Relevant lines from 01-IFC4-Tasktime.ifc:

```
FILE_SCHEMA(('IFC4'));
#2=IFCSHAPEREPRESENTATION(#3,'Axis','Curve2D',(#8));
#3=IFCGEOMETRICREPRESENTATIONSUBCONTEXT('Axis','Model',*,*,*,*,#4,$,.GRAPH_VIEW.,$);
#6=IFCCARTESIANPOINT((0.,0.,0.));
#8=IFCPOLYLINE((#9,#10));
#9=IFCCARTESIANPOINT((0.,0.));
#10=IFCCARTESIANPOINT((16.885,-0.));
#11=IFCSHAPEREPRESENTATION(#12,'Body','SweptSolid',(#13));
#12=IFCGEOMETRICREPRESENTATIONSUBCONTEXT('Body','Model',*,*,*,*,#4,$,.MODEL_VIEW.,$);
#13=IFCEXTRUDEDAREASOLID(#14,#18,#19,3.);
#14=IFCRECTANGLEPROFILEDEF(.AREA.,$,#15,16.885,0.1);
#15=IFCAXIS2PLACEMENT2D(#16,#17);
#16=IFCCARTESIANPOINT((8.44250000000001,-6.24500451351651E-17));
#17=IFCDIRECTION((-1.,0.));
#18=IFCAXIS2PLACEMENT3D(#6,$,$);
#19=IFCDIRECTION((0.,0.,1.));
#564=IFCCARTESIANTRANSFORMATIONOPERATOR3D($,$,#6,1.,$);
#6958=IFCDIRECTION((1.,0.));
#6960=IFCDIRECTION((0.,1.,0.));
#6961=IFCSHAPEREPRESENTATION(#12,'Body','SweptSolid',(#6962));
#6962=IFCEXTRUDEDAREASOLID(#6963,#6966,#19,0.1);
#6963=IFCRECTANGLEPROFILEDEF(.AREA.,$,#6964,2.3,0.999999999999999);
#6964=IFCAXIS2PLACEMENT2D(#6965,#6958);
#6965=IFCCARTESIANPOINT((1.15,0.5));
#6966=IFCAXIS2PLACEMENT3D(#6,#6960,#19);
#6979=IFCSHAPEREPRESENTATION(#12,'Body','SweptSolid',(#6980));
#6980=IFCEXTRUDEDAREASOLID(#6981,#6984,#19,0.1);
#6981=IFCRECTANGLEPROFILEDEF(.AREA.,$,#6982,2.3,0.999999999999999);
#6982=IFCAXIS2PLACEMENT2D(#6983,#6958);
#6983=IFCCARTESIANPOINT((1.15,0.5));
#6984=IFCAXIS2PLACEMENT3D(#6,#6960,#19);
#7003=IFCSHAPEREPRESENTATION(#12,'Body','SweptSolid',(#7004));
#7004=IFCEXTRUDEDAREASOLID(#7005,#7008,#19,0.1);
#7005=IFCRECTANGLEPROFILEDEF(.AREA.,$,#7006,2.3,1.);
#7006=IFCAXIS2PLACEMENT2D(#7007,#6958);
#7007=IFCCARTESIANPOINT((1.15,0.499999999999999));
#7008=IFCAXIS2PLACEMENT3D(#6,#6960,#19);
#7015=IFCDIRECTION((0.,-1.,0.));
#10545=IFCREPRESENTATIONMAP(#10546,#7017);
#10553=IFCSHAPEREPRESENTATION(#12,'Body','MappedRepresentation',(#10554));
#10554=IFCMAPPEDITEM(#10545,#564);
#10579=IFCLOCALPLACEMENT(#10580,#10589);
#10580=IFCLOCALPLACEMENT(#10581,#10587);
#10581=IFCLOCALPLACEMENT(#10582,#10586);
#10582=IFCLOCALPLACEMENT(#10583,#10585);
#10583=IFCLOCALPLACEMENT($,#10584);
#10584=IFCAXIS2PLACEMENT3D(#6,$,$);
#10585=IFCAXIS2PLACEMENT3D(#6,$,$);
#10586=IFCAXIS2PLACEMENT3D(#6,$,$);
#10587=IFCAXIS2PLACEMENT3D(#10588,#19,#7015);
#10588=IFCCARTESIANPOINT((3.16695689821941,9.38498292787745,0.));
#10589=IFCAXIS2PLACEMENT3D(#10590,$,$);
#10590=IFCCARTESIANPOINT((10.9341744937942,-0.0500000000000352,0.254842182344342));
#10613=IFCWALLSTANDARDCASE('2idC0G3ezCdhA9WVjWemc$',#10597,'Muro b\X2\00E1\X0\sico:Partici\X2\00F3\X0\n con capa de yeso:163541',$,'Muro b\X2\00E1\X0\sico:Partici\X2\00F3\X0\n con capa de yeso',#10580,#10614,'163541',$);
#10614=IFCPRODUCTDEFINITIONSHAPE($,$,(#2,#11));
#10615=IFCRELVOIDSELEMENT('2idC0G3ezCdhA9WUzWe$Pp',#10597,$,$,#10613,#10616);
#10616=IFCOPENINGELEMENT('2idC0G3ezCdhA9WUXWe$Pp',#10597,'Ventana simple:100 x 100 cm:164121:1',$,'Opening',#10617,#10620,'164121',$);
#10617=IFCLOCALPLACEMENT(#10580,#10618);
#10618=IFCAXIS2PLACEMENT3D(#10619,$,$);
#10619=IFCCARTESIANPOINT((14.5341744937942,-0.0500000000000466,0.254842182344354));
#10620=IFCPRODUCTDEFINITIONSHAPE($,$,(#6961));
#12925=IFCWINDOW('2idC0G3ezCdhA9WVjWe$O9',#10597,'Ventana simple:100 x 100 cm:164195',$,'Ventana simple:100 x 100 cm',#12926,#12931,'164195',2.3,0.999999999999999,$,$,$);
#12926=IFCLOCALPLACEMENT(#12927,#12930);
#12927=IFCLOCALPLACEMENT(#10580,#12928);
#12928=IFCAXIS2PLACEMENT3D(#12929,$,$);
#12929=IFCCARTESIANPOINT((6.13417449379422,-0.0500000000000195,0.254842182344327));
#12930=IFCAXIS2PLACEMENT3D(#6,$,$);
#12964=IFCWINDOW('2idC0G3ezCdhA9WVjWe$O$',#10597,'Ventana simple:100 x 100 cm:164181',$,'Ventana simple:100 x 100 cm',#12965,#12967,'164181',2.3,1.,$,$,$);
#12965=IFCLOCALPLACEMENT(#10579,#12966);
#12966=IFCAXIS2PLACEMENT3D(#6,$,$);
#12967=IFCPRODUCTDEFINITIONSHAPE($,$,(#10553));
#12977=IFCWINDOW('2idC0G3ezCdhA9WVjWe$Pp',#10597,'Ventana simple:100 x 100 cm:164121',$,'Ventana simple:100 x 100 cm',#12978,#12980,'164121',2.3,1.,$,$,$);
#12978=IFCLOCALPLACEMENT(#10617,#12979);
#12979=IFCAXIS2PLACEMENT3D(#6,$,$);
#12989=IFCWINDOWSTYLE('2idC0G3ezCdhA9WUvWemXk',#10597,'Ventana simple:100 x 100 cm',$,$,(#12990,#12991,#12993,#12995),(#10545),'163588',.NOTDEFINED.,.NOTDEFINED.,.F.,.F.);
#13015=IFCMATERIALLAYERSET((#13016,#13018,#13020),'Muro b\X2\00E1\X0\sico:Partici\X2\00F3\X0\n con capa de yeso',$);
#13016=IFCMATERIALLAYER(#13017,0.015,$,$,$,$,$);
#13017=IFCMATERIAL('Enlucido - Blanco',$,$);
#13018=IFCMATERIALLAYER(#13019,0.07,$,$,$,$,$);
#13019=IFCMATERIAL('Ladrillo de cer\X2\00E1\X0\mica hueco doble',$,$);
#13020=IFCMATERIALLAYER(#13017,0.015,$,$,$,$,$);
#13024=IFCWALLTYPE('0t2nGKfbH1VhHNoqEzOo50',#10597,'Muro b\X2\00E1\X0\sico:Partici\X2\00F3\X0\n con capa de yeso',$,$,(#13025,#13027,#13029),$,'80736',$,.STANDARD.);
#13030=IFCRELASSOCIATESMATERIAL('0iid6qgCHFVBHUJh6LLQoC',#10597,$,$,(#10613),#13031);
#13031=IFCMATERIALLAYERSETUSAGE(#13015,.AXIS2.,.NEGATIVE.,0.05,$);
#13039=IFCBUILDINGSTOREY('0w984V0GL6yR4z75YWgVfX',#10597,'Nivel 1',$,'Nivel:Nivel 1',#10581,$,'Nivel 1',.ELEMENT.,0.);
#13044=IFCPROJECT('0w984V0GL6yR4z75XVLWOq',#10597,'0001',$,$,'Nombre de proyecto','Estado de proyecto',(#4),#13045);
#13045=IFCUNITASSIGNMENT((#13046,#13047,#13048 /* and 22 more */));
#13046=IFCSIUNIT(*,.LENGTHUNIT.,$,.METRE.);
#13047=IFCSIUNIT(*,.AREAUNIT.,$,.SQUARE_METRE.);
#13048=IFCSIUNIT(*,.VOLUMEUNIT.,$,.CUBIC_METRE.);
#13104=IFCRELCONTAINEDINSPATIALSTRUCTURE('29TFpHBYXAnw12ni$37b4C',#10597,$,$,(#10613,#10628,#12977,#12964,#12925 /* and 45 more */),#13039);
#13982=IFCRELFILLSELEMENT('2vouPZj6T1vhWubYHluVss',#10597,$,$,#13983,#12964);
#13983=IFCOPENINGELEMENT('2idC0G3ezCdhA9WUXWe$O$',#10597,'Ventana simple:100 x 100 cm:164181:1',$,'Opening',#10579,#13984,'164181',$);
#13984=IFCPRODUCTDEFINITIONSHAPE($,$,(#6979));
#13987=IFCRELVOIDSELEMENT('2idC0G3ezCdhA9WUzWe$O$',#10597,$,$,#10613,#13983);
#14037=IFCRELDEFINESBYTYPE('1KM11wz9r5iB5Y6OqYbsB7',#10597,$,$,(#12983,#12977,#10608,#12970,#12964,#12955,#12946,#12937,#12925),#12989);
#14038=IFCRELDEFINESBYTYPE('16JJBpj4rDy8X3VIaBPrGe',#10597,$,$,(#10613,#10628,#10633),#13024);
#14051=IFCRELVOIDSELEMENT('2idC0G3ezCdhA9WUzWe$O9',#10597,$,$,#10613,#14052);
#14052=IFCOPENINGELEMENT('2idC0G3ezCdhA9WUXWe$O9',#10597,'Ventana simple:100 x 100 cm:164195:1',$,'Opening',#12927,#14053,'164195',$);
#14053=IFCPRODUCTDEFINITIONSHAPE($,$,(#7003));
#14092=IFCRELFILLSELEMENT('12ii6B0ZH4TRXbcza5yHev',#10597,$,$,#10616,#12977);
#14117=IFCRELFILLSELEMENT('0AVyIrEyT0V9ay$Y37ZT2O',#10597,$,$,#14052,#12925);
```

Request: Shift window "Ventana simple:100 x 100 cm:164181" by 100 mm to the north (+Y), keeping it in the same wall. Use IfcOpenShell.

```python
import ifcopenshell
import ifcopenshell.api.geometry
import ifcopenshell.util.placement

model = ifcopenshell.open("01-IFC4-Tasktime.ifc")

window = model.by_id(12964)
opening = window.FillsVoids[0].RelatingOpeningElement
wall = opening.VoidsElements[0].RelatingBuildingElement

wall_matrix = ifcopenshell.util.placement.get_local_placement(wall.ObjectPlacement)
shift = wall_matrix[:3, 0] * -0.1
before = ifcopenshell.util.placement.get_local_placement(window.ObjectPlacement)[:3, 3].copy()

# The window is placed relative to its opening, so it follows when the opening moves.
matrix = ifcopenshell.util.placement.get_local_placement(opening.ObjectPlacement)
matrix[:3, 3] += shift
ifcopenshell.api.geometry.edit_object_placement(
    model, product=opening, matrix=matrix, is_si=False, should_transform_children=True
)

after = ifcopenshell.util.placement.get_local_placement(window.ObjectPlacement)[:3, 3]
print("window moved by", (after - before).round(3) + 0.0)

model.write("01-IFC4-Tasktime_rev.ifc")
```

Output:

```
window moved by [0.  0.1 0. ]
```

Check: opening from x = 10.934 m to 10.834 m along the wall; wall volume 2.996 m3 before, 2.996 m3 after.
